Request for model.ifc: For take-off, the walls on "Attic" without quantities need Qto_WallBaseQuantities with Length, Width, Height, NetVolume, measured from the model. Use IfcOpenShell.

First a look at what the model holds.

```python
import ifcopenshell
import ifcopenshell.util.element
import ifcopenshell.util.unit

model = ifcopenshell.open("model.ifc")
print(model.schema)
for unit_type in ("LENGTHUNIT", "AREAUNIT", "VOLUMEUNIT"):
    print(unit_type, ifcopenshell.util.unit.calculate_unit_scale(model, unit_type))
storey = next(s for s in model.by_type("IfcBuildingStorey") if s.Name == "Attic")
walls = [e for e in ifcopenshell.util.element.get_decomposition(storey) if e.is_a("IfcWall")]
for e in sorted(walls, key=lambda e: e.id()):
    print(e.id(), e.is_a(), e.Name, list(ifcopenshell.util.element.get_psets(e, qtos_only=True)), sep=" | ")
```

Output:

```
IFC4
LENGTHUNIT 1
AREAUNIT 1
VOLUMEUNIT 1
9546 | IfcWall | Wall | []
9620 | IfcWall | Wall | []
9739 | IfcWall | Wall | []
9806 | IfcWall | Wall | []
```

```python
import ifcopenshell
import ifcopenshell.api.pset
import ifcopenshell.geom
import ifcopenshell.util.element
import ifcopenshell.util.shape
import ifcopenshell.util.unit

model = ifcopenshell.open("model.ifc")
unit_scale = ifcopenshell.util.unit.calculate_unit_scale(model)
volume_scale = ifcopenshell.util.unit.calculate_unit_scale(model, "VOLUMEUNIT")
settings = ifcopenshell.geom.settings()

storey = next(s for s in model.by_type("IfcBuildingStorey") if s.Name == "Attic")
walls = [e for e in ifcopenshell.util.element.get_decomposition(storey) if e.is_a("IfcWall")]

for e in sorted(walls, key=lambda e: e.id()):
    if ifcopenshell.util.element.get_psets(e, qtos_only=True, should_inherit=False):
        continue
    # Geometry comes back in metres, in the element's own axes.
    shape = ifcopenshell.geom.create_shape(settings, e)
    values = {
        "Length": ifcopenshell.util.shape.get_x(shape.geometry) / unit_scale,
        "Width": ifcopenshell.util.shape.get_y(shape.geometry) / unit_scale,
        "Height": ifcopenshell.util.shape.get_z(shape.geometry) / unit_scale,
        "NetVolume": ifcopenshell.util.shape.get_volume(shape.geometry) / volume_scale,
    }
    qto = ifcopenshell.api.pset.add_qto(model, product=e, name="Qto_WallBaseQuantities")
    ifcopenshell.api.pset.edit_qto(model, qto=qto, properties=values)
    print(e.id(), {k: round(v, 3) for k, v in values.items()})

model.write("model_rev.ifc")
```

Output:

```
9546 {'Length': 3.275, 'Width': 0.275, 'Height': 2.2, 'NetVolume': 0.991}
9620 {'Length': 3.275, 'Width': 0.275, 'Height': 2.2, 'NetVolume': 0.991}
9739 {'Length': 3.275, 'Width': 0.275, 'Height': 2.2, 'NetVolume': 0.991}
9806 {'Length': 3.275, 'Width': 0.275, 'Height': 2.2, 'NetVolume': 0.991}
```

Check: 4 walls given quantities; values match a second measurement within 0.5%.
